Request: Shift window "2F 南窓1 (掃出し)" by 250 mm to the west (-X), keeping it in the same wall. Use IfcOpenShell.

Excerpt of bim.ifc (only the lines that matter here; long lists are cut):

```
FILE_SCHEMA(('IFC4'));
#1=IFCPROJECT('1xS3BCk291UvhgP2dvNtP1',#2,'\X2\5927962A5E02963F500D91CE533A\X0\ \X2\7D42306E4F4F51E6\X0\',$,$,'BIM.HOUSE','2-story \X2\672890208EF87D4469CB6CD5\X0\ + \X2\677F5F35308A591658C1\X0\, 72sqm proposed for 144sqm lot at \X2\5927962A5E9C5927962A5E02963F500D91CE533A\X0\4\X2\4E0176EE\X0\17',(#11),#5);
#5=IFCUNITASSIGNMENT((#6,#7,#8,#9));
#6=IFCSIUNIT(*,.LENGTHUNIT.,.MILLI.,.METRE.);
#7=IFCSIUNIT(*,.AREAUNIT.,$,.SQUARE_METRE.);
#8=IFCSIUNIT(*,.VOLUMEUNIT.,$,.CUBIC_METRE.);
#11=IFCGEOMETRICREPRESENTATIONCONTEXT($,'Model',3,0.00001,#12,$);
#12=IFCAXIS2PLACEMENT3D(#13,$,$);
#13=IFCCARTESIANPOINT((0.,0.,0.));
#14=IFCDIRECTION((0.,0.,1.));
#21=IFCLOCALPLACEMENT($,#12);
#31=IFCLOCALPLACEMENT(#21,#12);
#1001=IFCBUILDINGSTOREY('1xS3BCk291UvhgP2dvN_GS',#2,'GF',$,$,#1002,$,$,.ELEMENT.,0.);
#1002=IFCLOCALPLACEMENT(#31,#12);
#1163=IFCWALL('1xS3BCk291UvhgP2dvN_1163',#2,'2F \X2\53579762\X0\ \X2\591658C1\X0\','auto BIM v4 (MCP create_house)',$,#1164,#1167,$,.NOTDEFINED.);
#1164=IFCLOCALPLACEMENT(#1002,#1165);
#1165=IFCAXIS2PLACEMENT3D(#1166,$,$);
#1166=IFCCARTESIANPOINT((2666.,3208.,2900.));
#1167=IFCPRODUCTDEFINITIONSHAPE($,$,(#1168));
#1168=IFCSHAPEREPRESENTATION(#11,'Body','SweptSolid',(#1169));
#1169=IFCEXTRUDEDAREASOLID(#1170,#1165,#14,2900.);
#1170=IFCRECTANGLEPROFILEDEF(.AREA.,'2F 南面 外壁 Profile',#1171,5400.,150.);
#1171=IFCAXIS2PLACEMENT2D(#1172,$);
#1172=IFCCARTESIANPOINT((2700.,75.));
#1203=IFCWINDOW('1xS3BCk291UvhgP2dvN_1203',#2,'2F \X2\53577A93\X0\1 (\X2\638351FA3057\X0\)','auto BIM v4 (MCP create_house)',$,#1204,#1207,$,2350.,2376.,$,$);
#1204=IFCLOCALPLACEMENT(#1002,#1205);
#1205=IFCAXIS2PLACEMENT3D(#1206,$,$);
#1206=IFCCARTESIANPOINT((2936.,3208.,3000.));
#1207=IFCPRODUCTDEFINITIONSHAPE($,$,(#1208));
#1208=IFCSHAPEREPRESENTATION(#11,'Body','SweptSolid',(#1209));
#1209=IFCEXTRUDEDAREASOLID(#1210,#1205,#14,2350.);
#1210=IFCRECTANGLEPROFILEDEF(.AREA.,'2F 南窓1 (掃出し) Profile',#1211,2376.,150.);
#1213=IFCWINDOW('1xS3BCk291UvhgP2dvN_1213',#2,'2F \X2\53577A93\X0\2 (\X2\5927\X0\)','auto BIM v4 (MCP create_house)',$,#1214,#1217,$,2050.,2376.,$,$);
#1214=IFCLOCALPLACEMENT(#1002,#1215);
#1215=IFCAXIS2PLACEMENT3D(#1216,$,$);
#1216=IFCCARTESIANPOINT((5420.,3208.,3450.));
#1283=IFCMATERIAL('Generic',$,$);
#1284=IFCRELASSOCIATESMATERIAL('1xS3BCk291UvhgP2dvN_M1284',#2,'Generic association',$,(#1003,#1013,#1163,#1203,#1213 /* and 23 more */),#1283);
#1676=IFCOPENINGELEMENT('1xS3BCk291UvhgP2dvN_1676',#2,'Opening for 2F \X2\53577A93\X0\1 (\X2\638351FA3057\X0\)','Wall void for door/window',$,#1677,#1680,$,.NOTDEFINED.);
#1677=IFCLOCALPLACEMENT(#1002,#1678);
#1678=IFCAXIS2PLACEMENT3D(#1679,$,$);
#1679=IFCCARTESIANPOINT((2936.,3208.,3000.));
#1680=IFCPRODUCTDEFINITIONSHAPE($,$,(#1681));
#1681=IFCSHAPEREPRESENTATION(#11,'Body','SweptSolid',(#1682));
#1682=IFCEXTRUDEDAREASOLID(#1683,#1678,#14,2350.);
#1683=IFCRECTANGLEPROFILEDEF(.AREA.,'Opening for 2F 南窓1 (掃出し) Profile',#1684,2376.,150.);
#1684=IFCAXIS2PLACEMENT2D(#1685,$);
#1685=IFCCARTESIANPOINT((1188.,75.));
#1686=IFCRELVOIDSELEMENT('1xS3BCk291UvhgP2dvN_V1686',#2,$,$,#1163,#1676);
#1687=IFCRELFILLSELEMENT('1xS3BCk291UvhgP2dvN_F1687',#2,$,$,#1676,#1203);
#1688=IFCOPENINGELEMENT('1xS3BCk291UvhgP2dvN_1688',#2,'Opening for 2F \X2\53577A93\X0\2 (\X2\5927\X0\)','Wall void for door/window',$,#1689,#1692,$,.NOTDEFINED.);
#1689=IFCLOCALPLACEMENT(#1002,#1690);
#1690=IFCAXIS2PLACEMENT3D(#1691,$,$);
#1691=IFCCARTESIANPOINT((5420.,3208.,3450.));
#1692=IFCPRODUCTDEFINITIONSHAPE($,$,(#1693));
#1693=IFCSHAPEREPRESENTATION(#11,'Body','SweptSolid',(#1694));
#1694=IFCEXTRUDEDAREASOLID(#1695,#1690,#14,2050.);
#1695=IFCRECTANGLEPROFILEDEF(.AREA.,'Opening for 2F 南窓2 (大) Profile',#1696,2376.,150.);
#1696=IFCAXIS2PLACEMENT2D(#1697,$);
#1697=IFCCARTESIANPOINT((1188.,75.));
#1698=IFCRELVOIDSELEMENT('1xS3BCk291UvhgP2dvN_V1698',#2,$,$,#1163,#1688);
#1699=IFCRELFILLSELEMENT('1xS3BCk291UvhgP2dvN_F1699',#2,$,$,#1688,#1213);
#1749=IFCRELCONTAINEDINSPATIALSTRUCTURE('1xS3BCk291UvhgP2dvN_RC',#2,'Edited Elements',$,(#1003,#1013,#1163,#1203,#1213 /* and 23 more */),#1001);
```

```python
import ifcopenshell
import ifcopenshell.api.geometry
import ifcopenshell.util.placement
import ifcopenshell.util.unit

model = ifcopenshell.open("bim.ifc")
unit_scale = ifcopenshell.util.unit.calculate_unit_scale(model)

window = model.by_id(1203)
opening = window.FillsVoids[0].RelatingOpeningElement
wall = opening.VoidsElements[0].RelatingBuildingElement

wall_matrix = ifcopenshell.util.placement.get_local_placement(wall.ObjectPlacement)
shift = wall_matrix[:3, 0] * -0.25 / unit_scale
before = ifcopenshell.util.placement.get_local_placement(window.ObjectPlacement)[:3, 3].copy()

# The window is not placed relative to its opening, so move both.
for product in (opening, window):
    matrix = ifcopenshell.util.placement.get_local_placement(product.ObjectPlacement)
    matrix[:3, 3] += shift
    ifcopenshell.api.geometry.edit_object_placement(model, product=product, matrix=matrix, is_si=False)

after = ifcopenshell.util.placement.get_local_placement(window.ObjectPlacement)[:3, 3]
print("window moved by", (after - before).round(3) + 0.0)

model.write("bim_v2.ifc")
```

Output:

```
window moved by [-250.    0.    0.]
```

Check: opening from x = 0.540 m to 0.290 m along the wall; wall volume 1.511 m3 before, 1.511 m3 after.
